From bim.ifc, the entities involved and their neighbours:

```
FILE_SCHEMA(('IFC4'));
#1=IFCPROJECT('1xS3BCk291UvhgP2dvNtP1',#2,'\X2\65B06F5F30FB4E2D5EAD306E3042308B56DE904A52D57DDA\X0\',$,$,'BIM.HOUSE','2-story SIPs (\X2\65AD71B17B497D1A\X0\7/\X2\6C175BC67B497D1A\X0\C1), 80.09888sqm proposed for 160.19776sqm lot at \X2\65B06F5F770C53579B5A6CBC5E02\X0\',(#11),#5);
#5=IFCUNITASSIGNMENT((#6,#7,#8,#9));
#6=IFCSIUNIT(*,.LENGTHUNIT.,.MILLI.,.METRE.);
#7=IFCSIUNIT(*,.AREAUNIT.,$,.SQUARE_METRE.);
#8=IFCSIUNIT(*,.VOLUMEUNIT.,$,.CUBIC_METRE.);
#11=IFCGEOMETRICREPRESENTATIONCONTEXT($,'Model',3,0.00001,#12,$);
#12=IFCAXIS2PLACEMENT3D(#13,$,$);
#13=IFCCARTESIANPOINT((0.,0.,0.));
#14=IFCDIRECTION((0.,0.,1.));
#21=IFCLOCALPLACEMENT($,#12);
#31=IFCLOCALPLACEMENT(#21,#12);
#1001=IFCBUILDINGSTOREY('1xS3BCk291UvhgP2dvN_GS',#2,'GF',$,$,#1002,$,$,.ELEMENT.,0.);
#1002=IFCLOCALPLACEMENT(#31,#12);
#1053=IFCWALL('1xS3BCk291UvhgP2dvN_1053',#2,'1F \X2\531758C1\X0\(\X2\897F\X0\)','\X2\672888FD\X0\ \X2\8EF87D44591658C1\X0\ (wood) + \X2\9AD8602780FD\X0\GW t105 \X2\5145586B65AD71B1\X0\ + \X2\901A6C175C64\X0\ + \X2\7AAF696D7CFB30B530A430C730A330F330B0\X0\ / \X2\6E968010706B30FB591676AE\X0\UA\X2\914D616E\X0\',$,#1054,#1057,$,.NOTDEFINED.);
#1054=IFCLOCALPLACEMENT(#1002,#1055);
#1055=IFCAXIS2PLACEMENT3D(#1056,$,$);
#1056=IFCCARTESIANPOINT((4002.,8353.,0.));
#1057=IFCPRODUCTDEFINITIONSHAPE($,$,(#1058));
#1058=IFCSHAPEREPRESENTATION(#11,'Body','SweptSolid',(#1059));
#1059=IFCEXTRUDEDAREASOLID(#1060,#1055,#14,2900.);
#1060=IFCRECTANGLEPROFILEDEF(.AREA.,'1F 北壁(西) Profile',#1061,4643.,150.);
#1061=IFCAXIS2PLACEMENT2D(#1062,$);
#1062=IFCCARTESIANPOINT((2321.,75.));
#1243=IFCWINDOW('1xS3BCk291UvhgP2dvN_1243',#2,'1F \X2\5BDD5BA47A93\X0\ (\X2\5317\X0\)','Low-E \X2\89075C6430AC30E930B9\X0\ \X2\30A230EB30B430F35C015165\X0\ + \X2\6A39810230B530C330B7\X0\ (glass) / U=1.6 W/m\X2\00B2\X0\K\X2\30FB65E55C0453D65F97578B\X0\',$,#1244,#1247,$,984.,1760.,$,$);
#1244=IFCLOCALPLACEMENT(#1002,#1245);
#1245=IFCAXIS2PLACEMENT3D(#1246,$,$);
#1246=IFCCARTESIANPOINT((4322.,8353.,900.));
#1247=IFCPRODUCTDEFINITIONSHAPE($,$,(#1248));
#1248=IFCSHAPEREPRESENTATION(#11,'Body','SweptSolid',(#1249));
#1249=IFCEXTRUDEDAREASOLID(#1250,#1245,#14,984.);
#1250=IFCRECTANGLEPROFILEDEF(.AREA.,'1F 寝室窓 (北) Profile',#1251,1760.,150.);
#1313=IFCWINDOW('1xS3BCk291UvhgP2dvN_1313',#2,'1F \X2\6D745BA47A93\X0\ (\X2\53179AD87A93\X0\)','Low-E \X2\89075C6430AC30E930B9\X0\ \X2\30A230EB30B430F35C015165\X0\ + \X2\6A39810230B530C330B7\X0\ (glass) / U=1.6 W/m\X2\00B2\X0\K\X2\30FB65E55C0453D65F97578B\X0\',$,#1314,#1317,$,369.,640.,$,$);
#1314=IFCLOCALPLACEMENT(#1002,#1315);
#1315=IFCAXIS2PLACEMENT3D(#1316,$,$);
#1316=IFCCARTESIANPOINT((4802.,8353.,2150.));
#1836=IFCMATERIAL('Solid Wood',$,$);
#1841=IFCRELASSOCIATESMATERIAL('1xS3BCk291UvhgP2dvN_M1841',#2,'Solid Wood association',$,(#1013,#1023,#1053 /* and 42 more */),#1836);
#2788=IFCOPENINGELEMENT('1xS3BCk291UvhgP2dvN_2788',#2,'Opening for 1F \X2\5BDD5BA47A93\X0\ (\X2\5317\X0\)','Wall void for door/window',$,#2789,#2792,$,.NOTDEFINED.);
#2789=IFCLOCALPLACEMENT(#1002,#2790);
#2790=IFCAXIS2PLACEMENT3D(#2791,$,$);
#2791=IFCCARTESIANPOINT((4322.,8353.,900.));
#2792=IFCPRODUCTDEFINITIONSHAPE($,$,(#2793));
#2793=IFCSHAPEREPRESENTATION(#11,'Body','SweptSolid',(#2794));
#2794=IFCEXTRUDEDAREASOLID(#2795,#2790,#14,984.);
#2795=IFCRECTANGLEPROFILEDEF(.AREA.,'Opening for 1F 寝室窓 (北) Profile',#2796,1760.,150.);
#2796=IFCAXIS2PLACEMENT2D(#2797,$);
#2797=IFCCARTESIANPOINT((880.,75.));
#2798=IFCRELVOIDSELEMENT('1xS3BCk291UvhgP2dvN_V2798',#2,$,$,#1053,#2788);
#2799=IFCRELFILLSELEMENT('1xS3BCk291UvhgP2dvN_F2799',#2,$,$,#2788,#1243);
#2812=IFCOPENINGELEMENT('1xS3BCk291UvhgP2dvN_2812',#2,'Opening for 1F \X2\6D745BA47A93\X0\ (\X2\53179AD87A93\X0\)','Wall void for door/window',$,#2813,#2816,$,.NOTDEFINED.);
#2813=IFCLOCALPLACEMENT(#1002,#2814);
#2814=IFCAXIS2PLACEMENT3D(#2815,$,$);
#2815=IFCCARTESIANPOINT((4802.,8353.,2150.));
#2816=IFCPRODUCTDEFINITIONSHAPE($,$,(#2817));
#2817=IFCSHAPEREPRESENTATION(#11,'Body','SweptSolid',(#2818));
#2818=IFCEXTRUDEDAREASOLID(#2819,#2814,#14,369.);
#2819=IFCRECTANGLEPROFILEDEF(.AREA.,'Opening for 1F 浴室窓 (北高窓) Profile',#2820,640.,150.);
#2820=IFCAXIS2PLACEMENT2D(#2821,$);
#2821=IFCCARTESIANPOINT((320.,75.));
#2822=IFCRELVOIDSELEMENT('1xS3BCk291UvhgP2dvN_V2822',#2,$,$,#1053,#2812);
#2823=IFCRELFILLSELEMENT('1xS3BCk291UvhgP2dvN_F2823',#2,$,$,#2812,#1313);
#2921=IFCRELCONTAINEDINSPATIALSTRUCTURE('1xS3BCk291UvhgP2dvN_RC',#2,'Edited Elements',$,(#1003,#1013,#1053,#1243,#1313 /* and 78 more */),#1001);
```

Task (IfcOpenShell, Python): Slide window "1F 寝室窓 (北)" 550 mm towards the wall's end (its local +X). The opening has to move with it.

```python
import ifcopenshell
import ifcopenshell.api.geometry
import ifcopenshell.util.placement

model = ifcopenshell.open("bim.ifc")

window = model.by_guid("1xS3BCk291UvhgP2dvN_1243")
opening = window.FillsVoids[0].RelatingOpeningElement
wall = opening.VoidsElements[0].RelatingBuildingElement

wall_matrix = ifcopenshell.util.placement.get_local_placement(wall.ObjectPlacement)
shift = wall_matrix[:3, 0] * 550.0
before = ifcopenshell.util.placement.get_local_placement(window.ObjectPlacement)[:3, 3].copy()

# The window is not placed relative to its opening, so move both.
for product in (opening, window):
    matrix = ifcopenshell.util.placement.get_local_placement(product.ObjectPlacement)
    matrix[:3, 3] += shift
    ifcopenshell.api.geometry.edit_object_placement(model, product=product, matrix=matrix, is_si=False)

after = ifcopenshell.util.placement.get_local_placement(window.ObjectPlacement)[:3, 3]
print("window moved by", (after - before).round(3) + 0.0)

model.write("bim_edited.ifc")
```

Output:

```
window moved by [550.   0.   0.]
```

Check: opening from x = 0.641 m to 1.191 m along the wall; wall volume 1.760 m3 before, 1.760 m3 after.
